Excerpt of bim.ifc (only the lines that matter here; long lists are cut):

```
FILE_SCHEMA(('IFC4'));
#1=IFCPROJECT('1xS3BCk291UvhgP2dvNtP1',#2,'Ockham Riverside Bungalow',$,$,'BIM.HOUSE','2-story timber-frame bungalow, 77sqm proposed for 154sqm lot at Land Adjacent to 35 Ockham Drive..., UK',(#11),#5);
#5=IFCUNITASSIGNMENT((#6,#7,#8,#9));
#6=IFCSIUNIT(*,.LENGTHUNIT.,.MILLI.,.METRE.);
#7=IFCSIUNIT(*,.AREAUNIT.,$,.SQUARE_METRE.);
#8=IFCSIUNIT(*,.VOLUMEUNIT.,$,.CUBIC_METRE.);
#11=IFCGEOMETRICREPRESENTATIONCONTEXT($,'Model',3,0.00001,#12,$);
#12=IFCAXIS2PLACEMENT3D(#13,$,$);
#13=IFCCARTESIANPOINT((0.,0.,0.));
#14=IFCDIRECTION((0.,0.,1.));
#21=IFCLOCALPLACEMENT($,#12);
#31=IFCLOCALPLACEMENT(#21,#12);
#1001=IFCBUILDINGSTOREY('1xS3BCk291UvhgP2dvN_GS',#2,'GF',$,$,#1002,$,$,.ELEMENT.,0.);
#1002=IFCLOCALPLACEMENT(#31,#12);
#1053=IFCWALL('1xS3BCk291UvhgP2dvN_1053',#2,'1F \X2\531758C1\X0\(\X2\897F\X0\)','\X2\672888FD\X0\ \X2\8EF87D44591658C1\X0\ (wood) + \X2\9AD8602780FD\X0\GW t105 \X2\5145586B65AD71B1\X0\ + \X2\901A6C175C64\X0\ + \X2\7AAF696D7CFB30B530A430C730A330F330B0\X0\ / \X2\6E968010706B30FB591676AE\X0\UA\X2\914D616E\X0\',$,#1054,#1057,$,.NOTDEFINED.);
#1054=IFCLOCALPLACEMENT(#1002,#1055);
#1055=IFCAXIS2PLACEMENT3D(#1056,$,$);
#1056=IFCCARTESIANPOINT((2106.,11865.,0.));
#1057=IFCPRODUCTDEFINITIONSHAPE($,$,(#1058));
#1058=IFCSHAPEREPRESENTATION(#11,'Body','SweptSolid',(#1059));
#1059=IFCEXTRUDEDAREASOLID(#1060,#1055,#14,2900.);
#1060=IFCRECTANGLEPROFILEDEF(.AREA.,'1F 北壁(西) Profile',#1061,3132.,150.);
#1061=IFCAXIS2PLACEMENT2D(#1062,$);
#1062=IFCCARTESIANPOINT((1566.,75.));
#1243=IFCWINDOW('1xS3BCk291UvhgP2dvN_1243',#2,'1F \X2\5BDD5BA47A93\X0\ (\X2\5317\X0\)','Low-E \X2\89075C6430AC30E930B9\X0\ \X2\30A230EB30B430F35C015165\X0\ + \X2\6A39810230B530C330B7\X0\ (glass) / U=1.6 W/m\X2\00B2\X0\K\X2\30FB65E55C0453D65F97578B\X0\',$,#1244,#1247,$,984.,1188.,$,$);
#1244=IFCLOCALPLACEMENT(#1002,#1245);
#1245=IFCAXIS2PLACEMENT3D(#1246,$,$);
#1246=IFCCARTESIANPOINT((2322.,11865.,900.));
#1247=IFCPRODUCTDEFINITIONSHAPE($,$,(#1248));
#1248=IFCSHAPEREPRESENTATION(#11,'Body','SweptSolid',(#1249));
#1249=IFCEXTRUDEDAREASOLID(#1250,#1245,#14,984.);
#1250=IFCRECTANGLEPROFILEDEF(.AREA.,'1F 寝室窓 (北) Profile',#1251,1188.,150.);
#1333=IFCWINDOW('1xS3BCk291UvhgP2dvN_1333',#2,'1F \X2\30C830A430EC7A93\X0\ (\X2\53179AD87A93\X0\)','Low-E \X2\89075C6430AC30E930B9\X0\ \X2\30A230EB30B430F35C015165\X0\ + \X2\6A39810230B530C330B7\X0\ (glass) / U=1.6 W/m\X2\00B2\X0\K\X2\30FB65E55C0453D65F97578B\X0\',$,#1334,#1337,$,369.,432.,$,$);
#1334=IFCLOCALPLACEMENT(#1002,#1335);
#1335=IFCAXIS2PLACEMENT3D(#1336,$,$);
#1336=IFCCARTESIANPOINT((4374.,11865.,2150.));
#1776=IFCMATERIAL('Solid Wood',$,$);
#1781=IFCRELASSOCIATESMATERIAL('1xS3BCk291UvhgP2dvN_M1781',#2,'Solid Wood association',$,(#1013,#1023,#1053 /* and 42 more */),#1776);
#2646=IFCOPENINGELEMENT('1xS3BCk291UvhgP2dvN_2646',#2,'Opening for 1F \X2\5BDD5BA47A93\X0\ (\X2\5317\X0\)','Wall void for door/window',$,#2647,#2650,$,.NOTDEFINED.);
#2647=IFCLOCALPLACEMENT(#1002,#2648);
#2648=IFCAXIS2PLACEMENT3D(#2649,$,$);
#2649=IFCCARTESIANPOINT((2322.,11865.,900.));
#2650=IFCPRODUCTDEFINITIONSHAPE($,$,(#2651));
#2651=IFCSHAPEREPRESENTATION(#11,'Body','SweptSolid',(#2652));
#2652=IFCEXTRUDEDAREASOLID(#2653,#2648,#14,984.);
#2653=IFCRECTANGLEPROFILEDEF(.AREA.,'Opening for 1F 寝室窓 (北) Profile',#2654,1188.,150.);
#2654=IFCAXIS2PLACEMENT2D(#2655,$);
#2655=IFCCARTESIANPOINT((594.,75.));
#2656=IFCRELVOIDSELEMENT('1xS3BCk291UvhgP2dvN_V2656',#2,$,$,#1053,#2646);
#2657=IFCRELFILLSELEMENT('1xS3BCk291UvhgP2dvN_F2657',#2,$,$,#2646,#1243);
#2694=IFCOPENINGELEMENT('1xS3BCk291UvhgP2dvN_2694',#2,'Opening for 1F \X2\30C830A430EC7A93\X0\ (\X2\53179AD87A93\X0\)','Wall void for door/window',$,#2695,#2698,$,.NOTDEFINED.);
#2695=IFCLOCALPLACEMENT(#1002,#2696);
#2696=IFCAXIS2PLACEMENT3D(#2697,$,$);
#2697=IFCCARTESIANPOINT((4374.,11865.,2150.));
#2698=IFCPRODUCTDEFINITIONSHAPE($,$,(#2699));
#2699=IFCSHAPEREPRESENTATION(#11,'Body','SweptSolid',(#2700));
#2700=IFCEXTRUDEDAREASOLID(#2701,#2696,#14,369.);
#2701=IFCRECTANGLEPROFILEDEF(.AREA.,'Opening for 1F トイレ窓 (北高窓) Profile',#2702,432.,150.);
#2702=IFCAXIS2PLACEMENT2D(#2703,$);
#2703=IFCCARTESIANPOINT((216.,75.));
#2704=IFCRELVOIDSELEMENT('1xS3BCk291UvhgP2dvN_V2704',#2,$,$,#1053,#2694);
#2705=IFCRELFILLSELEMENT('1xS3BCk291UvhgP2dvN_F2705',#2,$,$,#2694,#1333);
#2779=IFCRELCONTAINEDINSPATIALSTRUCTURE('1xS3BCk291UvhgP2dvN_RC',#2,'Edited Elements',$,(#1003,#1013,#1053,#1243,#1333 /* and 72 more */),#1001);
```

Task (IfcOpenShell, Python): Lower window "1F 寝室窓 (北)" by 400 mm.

```python
import numpy as np
import ifcopenshell
import ifcopenshell.api.geometry
import ifcopenshell.util.placement
import ifcopenshell.util.unit

model = ifcopenshell.open("bim.ifc")
unit_scale = ifcopenshell.util.unit.calculate_unit_scale(model)

window = model.by_guid("1xS3BCk291UvhgP2dvN_1243")
opening = window.FillsVoids[0].RelatingOpeningElement
dz = -0.4 / unit_scale

shift = np.array([0.0, 0.0, dz])
# The window is not placed relative to its opening, so move both.
for product in (opening, window):
    matrix = ifcopenshell.util.placement.get_local_placement(product.ObjectPlacement)
    matrix[:3, 3] += shift
    ifcopenshell.api.geometry.edit_object_placement(model, product=product, matrix=matrix, is_si=False)

print(f"moved by {dz * unit_scale:+.3f} m")

model.write("bim_rev.ifc")
```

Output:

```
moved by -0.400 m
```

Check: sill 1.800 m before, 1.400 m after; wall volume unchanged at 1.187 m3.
